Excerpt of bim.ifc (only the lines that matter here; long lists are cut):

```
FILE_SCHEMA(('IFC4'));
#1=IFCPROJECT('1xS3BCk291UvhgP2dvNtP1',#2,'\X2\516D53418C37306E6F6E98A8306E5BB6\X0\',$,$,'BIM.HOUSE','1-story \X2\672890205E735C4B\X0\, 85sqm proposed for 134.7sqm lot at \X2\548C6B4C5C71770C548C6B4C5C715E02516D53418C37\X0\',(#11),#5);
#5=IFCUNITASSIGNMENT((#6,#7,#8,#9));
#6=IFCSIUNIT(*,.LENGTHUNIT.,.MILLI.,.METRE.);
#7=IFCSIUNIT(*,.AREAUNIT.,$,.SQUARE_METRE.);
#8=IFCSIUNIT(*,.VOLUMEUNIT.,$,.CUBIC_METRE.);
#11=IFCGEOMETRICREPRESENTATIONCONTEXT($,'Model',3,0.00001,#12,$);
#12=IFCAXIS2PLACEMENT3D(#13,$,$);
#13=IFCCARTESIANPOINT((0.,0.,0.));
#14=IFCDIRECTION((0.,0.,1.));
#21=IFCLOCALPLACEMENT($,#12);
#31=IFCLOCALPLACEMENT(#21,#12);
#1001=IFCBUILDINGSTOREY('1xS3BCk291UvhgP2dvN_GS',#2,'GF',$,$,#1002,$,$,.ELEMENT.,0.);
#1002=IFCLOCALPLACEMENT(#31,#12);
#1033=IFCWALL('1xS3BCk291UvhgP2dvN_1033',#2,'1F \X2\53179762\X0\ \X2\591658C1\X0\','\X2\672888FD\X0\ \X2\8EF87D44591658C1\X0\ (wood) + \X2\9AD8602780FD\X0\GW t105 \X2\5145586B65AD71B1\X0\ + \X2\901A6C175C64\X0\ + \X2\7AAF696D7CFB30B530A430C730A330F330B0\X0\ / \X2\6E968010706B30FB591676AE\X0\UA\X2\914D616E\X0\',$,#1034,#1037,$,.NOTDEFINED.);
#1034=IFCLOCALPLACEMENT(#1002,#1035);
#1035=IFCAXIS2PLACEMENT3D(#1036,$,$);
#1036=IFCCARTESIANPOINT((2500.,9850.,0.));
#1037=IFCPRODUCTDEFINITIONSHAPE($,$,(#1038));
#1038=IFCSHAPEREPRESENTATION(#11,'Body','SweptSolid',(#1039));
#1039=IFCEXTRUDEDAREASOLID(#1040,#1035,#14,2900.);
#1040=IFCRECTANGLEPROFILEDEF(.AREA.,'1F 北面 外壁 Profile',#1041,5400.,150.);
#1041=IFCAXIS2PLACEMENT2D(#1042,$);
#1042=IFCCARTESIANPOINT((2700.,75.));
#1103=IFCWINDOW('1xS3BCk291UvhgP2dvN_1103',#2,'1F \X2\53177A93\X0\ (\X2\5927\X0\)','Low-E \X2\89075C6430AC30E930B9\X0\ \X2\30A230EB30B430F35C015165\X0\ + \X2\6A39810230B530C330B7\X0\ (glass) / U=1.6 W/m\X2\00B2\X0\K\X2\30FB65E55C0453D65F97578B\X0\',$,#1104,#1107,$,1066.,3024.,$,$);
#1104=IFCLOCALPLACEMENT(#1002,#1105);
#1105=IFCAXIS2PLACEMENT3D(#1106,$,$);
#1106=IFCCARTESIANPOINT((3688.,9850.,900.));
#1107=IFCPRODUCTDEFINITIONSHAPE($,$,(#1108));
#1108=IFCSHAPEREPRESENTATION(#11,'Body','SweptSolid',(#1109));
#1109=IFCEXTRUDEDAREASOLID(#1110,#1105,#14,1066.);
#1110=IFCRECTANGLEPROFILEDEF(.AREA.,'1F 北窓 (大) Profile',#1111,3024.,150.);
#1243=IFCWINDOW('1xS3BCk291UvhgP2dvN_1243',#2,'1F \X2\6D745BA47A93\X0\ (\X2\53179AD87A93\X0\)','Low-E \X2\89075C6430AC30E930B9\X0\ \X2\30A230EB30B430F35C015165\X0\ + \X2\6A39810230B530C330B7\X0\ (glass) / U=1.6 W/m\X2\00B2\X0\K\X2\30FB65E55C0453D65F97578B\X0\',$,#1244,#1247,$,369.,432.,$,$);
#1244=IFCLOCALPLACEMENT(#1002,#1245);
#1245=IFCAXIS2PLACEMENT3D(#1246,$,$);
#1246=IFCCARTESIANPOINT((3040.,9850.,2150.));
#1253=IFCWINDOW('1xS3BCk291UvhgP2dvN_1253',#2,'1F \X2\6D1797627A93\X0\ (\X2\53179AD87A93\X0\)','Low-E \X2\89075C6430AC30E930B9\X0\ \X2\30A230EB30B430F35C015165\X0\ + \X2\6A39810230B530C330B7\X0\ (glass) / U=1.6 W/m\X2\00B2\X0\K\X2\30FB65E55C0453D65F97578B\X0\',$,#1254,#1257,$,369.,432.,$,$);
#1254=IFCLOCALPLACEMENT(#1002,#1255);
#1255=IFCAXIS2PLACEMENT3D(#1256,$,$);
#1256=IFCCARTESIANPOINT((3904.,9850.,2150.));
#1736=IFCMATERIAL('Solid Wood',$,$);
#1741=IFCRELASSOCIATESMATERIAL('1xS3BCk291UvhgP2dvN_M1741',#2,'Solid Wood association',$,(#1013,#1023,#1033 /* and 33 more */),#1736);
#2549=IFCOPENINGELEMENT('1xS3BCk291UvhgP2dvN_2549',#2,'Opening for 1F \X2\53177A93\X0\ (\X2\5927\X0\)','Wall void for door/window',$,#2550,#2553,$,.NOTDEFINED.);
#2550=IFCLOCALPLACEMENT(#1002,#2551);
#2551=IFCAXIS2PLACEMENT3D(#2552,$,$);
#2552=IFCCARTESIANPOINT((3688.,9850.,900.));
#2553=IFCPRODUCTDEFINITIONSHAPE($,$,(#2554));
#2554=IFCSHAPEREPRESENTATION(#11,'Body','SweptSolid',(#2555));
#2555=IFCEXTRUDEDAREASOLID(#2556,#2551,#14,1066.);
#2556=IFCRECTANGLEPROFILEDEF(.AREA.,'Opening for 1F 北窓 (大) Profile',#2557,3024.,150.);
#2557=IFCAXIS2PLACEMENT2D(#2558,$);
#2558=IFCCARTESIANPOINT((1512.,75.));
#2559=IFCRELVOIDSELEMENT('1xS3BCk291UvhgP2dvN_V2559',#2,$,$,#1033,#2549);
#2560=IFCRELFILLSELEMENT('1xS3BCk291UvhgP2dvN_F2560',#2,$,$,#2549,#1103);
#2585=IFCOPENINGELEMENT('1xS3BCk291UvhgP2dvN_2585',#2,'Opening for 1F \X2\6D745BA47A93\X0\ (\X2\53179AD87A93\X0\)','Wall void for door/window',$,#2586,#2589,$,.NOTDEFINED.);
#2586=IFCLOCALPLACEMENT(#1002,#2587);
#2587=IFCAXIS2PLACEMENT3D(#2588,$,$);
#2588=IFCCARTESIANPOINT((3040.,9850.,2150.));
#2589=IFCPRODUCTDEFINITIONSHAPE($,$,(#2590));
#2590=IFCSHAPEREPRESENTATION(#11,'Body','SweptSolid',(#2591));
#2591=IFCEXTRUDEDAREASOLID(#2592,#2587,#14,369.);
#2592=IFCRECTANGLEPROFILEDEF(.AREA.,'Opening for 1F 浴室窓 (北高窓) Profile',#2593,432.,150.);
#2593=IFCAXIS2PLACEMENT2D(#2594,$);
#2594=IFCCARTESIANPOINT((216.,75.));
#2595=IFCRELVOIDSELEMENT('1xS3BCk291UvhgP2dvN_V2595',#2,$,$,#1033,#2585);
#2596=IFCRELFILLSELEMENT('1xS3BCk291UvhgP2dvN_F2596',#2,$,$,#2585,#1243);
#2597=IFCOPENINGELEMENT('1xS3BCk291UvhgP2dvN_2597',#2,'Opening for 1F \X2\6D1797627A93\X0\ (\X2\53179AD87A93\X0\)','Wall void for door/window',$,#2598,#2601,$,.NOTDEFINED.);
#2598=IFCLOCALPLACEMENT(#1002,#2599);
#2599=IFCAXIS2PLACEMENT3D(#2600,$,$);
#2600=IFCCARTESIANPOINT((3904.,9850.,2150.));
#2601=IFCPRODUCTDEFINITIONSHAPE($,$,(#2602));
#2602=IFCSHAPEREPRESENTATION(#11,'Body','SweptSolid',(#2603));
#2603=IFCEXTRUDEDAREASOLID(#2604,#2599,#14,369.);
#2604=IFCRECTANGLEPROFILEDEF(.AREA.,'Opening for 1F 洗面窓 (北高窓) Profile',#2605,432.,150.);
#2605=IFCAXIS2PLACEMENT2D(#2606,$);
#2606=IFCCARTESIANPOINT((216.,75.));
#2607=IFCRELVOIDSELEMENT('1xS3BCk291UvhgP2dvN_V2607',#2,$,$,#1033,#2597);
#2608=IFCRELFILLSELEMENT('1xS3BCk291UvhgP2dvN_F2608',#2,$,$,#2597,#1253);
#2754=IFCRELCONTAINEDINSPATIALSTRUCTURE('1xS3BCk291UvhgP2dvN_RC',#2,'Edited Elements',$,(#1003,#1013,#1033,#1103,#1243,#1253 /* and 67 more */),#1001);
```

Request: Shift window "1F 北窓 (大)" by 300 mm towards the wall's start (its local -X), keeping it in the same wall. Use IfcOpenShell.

```python
import ifcopenshell
import ifcopenshell.api.geometry
import ifcopenshell.util.placement
import ifcopenshell.util.unit

model = ifcopenshell.open("bim.ifc")
unit_scale = ifcopenshell.util.unit.calculate_unit_scale(model)

window = model.by_guid("1xS3BCk291UvhgP2dvN_1103")
opening = window.FillsVoids[0].RelatingOpeningElement
wall = opening.VoidsElements[0].RelatingBuildingElement

wall_matrix = ifcopenshell.util.placement.get_local_placement(wall.ObjectPlacement)
shift = wall_matrix[:3, 0] * -0.3 / unit_scale
before = ifcopenshell.util.placement.get_local_placement(window.ObjectPlacement)[:3, 3].copy()

# The window is not placed relative to its opening, so move both.
for product in (opening, window):
    matrix = ifcopenshell.util.placement.get_local_placement(product.ObjectPlacement)
    matrix[:3, 3] += shift
    ifcopenshell.api.geometry.edit_object_placement(model, product=product, matrix=matrix, is_si=False)

after = ifcopenshell.util.placement.get_local_placement(window.ObjectPlacement)[:3, 3]
print("window moved by", (after - before).round(3) + 0.0)

model.write("bim_edited.ifc")
```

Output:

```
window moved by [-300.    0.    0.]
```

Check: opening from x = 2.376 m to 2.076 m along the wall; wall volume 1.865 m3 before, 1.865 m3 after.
